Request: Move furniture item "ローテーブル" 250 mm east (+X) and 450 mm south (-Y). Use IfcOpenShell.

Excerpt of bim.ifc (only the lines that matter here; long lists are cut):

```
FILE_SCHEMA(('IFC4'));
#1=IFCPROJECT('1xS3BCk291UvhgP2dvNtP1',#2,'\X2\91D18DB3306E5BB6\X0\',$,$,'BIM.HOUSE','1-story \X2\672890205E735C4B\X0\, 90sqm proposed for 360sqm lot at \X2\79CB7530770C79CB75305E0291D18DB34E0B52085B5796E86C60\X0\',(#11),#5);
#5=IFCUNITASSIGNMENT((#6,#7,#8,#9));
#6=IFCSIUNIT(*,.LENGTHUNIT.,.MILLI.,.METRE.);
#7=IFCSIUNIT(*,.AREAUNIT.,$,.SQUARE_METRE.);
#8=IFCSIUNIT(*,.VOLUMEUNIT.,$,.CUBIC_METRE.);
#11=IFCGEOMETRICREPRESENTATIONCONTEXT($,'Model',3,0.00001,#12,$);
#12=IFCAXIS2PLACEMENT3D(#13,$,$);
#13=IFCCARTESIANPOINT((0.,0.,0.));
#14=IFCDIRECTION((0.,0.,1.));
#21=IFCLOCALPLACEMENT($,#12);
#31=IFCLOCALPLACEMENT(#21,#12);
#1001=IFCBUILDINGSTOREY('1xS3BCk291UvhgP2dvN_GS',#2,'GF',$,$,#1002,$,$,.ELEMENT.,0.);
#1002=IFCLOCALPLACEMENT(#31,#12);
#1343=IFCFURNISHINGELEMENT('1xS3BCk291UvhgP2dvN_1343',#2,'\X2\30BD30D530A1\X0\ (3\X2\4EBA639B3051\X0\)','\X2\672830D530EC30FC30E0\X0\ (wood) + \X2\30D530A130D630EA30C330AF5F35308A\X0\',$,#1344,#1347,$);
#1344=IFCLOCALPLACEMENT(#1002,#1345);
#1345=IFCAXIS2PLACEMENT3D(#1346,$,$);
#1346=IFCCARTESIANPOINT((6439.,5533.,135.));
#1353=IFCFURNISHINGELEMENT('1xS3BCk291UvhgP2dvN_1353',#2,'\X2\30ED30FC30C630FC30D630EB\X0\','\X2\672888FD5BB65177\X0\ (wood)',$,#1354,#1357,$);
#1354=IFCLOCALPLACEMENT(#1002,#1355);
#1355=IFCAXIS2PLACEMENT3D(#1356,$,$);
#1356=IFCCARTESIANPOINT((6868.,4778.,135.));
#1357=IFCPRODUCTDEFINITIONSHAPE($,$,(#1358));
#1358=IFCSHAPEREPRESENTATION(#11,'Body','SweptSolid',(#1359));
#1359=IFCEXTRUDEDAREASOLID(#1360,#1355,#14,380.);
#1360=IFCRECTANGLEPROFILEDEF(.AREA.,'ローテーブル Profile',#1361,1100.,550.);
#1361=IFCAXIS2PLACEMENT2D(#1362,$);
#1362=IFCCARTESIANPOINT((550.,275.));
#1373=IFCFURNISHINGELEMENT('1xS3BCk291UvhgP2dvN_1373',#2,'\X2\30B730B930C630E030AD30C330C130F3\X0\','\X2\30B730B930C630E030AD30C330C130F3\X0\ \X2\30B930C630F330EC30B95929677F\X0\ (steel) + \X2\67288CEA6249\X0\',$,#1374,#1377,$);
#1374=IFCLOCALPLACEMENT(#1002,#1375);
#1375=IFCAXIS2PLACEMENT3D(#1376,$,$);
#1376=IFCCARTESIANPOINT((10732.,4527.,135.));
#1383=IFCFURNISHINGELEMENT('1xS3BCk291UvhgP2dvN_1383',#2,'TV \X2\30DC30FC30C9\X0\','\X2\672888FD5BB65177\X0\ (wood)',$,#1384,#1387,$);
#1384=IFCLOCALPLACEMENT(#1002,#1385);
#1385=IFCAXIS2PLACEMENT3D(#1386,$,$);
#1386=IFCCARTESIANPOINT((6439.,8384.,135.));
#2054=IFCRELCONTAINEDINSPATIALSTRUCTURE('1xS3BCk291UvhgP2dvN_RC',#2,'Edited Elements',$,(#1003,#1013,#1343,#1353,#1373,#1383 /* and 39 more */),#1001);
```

```python
import ifcopenshell
import ifcopenshell.api.geometry
import ifcopenshell.util.placement

model = ifcopenshell.open("bim.ifc")

item = model.by_guid("1xS3BCk291UvhgP2dvN_1353")
matrix = ifcopenshell.util.placement.get_local_placement(item.ObjectPlacement)
matrix[0, 3] += 250.0
matrix[1, 3] -= 450.0
ifcopenshell.api.geometry.edit_object_placement(model, product=item, matrix=matrix, is_si=False)

print(ifcopenshell.util.placement.get_local_placement(item.ObjectPlacement).round(3) + 0.0)

model.write("bim-out.ifc")
```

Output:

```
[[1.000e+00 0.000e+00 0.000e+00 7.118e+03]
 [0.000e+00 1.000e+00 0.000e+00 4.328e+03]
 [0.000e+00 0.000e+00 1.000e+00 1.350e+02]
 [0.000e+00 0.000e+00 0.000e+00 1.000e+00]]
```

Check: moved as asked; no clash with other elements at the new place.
